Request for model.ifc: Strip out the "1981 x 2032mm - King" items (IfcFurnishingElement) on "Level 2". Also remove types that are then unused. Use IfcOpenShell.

First a look at what the model holds.

```python
import ifcopenshell
import ifcopenshell.util.element

model = ifcopenshell.open("model.ifc")
print(model.schema)
storey = next(s for s in model.by_type("IfcBuildingStorey") if s.Name == "Level 2")
furniture = [e for e in ifcopenshell.util.element.get_decomposition(storey) if e.is_a("IfcFurnishingElement")]
seen = {}
for e in furniture:
    element_type = ifcopenshell.util.element.get_type(e)
    name = element_type.Name if element_type not in (None, e) else None
    seen[name] = seen.get(name, 0) + 1
for name, count in sorted(seen.items(), key=str):
    print(count, "x", name)
```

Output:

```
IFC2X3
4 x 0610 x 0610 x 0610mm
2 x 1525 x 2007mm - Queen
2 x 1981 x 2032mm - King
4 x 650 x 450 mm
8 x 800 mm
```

```python
import ifcopenshell
import ifcopenshell.api.root
import ifcopenshell.util.element

model = ifcopenshell.open("model.ifc")

storey = next(s for s in model.by_type("IfcBuildingStorey") if s.Name == "Level 2")
furniture = [e for e in ifcopenshell.util.element.get_decomposition(storey) if e.is_a("IfcFurnishingElement")]
targets = [e for e in furniture if (t := ifcopenshell.util.element.get_type(e)) not in (None, e) and t.Name == "1981 x 2032mm - King"]
types = {ifcopenshell.util.element.get_type(e) for e in targets} - {None, *targets}

for e in targets:
    ifcopenshell.api.root.remove_product(model, product=e)
print(len(targets), "removed")

unused = [t for t in types if not ifcopenshell.util.element.get_types(t)]
for t in unused:
    ifcopenshell.api.root.remove_product(model, product=t)
print(len(unused), "unused types removed")

model.write("model_rev.ifc")
```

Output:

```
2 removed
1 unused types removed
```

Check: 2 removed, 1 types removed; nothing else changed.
